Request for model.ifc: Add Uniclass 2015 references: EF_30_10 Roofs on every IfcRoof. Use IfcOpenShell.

First a look at what the model holds.

```python
import ifcopenshell

model = ifcopenshell.open("model.ifc")
print(model.schema)
print("classifications:", [c.Name for c in model.by_type("IfcClassification")])
for ifc_class in ("IfcDoor", "IfcRoof", "IfcStair", "IfcWall", "IfcWindow"):
    print(ifc_class, len(model.by_type(ifc_class)))
```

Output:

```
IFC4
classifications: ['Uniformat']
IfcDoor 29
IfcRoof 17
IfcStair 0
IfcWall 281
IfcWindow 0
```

```python
import ifcopenshell
import ifcopenshell.api.classification

model = ifcopenshell.open("model.ifc")

system = ifcopenshell.api.classification.add_classification(model, classification="Uniclass 2015")

codes = {
    "IfcRoof": ("EF_30_10", "Roofs"),
}
for ifc_class, (code, name) in codes.items():
    products = model.by_type(ifc_class)
    ifcopenshell.api.classification.add_reference(
        model, products=products, classification=system, identification=code, name=name
    )
    print(code, len(products))

model.write("model_rev.ifc")
```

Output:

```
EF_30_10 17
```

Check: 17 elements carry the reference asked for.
